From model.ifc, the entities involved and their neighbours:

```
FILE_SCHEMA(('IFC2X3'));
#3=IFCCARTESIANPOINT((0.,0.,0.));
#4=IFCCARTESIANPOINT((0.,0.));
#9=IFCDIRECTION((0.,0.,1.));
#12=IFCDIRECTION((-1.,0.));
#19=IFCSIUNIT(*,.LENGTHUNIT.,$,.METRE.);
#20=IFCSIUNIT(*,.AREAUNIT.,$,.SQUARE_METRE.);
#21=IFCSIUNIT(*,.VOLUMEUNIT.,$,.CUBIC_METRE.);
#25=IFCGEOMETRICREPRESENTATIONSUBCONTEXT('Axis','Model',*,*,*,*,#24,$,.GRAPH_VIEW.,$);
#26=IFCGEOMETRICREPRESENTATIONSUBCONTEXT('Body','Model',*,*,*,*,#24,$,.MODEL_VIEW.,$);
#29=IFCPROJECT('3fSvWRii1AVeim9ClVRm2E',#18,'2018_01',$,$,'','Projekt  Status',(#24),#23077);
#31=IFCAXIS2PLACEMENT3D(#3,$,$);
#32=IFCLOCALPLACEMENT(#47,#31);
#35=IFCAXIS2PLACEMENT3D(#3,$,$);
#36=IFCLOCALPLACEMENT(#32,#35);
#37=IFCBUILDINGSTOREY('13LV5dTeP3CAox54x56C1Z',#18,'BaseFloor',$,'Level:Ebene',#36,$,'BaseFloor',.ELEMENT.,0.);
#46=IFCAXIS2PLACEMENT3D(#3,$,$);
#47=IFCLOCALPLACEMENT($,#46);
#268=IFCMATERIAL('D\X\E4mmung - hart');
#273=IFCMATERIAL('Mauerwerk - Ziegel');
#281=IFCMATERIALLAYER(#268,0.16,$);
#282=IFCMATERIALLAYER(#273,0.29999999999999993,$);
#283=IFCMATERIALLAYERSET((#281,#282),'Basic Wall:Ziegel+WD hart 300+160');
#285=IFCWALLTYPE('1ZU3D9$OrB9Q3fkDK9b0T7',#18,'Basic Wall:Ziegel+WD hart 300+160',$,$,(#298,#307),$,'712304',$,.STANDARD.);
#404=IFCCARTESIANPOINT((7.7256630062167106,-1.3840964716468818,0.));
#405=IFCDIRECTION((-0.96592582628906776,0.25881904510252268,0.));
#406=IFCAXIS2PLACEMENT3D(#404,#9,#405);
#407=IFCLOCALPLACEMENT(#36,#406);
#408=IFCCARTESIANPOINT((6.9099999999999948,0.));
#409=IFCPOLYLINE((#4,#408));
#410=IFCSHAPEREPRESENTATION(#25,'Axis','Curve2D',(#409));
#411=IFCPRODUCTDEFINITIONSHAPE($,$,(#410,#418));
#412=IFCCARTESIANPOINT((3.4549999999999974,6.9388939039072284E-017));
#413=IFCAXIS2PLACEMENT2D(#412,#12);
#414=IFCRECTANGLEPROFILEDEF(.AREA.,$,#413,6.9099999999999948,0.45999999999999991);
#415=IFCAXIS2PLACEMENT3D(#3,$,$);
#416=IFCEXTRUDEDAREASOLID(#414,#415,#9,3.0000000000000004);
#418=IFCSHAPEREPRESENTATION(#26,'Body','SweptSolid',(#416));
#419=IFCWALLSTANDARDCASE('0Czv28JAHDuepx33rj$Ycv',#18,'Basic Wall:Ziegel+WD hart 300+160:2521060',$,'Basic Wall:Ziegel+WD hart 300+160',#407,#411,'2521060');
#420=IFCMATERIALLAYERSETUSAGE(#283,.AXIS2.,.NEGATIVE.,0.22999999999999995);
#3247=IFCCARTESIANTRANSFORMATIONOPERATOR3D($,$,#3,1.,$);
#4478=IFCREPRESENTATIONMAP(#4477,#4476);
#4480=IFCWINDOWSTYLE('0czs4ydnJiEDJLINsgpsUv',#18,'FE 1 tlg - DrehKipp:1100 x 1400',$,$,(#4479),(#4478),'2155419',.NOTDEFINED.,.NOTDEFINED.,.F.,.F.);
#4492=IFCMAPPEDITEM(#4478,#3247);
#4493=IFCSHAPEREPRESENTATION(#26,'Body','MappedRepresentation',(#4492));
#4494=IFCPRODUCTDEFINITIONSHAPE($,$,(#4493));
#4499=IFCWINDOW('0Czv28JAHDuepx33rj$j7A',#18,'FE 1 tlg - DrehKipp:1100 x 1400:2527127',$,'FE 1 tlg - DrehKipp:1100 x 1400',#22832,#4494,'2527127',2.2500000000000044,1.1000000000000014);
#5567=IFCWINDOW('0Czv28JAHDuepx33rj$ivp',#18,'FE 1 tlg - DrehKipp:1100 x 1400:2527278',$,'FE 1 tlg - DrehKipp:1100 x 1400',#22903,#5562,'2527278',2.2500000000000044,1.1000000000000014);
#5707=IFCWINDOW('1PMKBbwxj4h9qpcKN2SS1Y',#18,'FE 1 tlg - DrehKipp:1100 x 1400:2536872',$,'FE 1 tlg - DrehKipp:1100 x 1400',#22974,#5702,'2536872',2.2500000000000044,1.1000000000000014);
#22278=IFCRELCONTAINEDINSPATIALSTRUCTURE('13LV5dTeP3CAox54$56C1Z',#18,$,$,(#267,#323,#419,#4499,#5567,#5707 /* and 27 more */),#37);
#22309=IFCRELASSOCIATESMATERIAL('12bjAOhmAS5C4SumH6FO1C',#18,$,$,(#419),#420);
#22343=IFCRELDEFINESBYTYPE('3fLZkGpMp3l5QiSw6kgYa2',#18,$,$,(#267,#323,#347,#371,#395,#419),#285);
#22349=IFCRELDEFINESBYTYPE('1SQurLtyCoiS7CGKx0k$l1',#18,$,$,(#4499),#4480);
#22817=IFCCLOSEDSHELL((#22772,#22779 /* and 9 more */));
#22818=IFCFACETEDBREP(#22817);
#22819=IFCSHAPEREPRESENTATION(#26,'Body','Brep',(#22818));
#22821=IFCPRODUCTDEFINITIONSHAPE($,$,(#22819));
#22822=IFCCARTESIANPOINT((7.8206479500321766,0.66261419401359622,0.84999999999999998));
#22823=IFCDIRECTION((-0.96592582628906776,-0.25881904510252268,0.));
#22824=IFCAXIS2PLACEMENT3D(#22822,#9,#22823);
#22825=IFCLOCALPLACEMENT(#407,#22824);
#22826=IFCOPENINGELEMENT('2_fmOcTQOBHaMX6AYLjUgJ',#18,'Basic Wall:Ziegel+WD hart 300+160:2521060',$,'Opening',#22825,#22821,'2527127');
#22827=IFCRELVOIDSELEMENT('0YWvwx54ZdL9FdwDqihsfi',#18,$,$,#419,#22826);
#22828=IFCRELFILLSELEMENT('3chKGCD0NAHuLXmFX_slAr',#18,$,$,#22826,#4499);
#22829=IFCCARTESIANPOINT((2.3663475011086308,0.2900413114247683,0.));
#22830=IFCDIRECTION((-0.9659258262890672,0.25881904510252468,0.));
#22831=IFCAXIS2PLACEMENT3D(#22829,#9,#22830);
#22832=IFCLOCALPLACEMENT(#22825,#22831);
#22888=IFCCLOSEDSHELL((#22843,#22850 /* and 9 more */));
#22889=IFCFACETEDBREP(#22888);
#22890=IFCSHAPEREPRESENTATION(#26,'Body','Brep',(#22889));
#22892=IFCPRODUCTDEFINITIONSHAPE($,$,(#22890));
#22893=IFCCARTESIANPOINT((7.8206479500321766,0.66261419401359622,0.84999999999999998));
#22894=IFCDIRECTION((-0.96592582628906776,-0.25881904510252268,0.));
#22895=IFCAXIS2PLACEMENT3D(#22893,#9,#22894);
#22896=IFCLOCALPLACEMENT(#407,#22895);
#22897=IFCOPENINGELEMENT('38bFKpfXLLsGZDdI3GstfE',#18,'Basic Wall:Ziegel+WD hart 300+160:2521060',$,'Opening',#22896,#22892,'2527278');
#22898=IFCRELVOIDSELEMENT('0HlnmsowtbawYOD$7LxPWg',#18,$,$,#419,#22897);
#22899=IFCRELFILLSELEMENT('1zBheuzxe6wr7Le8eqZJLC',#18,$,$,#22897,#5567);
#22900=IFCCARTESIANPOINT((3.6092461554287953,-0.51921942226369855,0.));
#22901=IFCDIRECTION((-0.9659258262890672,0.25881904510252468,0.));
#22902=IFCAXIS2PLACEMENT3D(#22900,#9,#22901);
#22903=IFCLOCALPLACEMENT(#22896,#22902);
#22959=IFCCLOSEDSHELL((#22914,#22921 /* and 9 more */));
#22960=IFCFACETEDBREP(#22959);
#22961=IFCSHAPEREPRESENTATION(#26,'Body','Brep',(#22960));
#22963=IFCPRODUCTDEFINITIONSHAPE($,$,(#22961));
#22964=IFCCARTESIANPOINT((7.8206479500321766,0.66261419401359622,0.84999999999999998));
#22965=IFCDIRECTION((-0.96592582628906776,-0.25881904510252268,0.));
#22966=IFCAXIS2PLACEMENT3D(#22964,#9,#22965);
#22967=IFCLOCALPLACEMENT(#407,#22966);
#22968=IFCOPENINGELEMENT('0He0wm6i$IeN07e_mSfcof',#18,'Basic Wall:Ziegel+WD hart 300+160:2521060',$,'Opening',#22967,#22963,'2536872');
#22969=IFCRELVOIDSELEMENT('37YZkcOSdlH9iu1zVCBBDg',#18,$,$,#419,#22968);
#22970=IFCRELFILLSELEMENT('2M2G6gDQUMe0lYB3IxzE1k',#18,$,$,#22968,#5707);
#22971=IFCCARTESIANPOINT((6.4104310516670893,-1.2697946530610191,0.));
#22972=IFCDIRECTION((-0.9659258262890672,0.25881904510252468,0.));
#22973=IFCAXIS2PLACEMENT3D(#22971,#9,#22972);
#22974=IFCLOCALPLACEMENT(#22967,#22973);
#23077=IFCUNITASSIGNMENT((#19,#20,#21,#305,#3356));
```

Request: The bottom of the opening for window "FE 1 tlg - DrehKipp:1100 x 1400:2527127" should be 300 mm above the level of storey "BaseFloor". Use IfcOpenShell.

```python
import numpy as np
import ifcopenshell
import ifcopenshell.api.geometry
import ifcopenshell.geom
import ifcopenshell.util.element
import ifcopenshell.util.placement
import ifcopenshell.util.shape
import ifcopenshell.util.unit

model = ifcopenshell.open("model.ifc")
unit_scale = ifcopenshell.util.unit.calculate_unit_scale(model)

window = model.by_id(4499)
opening = window.FillsVoids[0].RelatingOpeningElement
storey = ifcopenshell.util.element.get_container(window, ifc_class="IfcBuildingStorey")
level = ifcopenshell.util.placement.get_local_placement(storey.ObjectPlacement)[2, 3]

# The opening's origin need not be at the sill, so measure its lowest point.
shape = ifcopenshell.geom.create_shape(ifcopenshell.geom.settings(), opening)
bottom = ifcopenshell.util.shape.get_shape_bottom_elevation(shape, shape.geometry) / unit_scale
dz = level + 0.3 - bottom

shift = np.array([0.0, 0.0, dz])
# The window is placed relative to its opening, so it follows when the opening moves.
matrix = ifcopenshell.util.placement.get_local_placement(opening.ObjectPlacement)
matrix[:3, 3] += shift
ifcopenshell.api.geometry.edit_object_placement(
    model, product=opening, matrix=matrix, is_si=False, should_transform_children=True
)

print(f"moved by {dz * unit_scale:+.3f} m")

model.write("model_rev.ifc")
```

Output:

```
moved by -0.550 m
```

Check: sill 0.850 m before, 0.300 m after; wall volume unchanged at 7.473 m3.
